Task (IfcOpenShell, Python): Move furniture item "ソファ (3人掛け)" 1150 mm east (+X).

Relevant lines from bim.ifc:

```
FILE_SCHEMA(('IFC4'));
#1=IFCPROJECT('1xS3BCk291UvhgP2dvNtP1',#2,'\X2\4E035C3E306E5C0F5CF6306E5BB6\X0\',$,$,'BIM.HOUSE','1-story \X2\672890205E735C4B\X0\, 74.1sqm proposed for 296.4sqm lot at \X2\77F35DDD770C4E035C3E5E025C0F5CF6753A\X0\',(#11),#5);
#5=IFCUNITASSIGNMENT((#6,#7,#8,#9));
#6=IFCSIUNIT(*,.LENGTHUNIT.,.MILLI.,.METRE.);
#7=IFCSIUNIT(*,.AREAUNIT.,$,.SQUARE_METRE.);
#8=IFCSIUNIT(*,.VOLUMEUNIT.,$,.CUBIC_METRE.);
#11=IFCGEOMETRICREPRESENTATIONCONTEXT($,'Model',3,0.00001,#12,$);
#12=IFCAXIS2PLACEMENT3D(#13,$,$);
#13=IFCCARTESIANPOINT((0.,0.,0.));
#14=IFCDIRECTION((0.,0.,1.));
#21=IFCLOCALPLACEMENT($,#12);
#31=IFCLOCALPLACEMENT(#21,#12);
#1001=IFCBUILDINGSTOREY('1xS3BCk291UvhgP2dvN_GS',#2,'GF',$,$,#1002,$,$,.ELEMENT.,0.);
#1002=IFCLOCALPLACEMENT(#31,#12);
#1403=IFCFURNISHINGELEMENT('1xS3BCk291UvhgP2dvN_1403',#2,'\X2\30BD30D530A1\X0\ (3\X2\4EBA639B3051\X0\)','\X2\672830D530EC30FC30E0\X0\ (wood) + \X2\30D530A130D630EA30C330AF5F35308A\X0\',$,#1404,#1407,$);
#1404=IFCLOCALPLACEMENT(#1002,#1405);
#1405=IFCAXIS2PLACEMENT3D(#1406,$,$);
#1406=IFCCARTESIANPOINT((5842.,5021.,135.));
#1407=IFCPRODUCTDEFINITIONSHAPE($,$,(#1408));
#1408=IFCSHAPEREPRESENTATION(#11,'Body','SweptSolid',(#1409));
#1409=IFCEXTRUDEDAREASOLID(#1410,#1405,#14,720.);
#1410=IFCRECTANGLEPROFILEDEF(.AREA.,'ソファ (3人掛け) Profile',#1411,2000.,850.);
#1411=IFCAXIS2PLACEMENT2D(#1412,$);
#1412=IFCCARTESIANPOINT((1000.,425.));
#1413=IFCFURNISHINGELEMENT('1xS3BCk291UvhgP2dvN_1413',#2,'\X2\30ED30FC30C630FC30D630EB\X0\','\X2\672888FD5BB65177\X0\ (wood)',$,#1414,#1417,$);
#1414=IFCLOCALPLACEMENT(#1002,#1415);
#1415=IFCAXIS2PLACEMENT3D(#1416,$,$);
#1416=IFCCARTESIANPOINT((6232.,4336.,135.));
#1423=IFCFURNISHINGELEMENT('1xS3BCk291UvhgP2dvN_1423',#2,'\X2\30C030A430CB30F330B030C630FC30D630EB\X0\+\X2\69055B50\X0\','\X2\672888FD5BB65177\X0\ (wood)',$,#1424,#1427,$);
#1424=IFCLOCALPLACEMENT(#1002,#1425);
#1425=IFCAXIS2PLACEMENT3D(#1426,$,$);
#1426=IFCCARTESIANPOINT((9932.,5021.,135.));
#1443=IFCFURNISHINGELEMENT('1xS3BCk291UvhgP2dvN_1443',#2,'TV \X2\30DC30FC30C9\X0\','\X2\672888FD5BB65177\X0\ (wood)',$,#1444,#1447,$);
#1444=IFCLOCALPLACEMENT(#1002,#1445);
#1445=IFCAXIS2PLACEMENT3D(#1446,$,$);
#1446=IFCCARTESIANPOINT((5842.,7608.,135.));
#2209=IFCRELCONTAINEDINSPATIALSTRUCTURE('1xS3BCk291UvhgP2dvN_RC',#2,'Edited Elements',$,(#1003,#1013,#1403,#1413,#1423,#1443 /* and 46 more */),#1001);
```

```python
import ifcopenshell
import ifcopenshell.api.geometry
import ifcopenshell.util.placement
import ifcopenshell.util.unit

model = ifcopenshell.open("bim.ifc")
unit_scale = ifcopenshell.util.unit.calculate_unit_scale(model)

item = model.by_guid("1xS3BCk291UvhgP2dvN_1403")
matrix = ifcopenshell.util.placement.get_local_placement(item.ObjectPlacement)
matrix[0, 3] += 1.15 / unit_scale
ifcopenshell.api.geometry.edit_object_placement(model, product=item, matrix=matrix, is_si=False)

print(ifcopenshell.util.placement.get_local_placement(item.ObjectPlacement).round(3) + 0.0)

model.write("bim_edited.ifc")
```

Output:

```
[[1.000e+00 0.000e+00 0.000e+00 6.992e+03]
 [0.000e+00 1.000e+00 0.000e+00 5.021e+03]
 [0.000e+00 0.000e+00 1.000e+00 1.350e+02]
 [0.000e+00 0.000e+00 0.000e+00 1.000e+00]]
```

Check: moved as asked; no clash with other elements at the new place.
